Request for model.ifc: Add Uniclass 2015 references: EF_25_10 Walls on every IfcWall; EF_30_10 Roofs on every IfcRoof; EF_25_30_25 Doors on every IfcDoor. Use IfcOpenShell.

First a look at what the model holds.

```python
import ifcopenshell

model = ifcopenshell.open("model.ifc")
print(model.schema)
print("classifications:", [c.Name for c in model.by_type("IfcClassification")])
for ifc_class in ("IfcDoor", "IfcRoof", "IfcStair", "IfcWall", "IfcWindow"):
    print(ifc_class, len(model.by_type(ifc_class)))
```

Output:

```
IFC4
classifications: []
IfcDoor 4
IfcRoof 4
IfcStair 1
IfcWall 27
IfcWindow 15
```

```python
import ifcopenshell
import ifcopenshell.api.classification

model = ifcopenshell.open("model.ifc")

system = ifcopenshell.api.classification.add_classification(model, classification="Uniclass 2015")

codes = {
    "IfcWall": ("EF_25_10", "Walls"),
    "IfcRoof": ("EF_30_10", "Roofs"),
    "IfcDoor": ("EF_25_30_25", "Doors"),
}
for ifc_class, (code, name) in codes.items():
    products = model.by_type(ifc_class)
    ifcopenshell.api.classification.add_reference(
        model, products=products, classification=system, identification=code, name=name
    )
    print(code, len(products))

model.write("model_v2.ifc")
```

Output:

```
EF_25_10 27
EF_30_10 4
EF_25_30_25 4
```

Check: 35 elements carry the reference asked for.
